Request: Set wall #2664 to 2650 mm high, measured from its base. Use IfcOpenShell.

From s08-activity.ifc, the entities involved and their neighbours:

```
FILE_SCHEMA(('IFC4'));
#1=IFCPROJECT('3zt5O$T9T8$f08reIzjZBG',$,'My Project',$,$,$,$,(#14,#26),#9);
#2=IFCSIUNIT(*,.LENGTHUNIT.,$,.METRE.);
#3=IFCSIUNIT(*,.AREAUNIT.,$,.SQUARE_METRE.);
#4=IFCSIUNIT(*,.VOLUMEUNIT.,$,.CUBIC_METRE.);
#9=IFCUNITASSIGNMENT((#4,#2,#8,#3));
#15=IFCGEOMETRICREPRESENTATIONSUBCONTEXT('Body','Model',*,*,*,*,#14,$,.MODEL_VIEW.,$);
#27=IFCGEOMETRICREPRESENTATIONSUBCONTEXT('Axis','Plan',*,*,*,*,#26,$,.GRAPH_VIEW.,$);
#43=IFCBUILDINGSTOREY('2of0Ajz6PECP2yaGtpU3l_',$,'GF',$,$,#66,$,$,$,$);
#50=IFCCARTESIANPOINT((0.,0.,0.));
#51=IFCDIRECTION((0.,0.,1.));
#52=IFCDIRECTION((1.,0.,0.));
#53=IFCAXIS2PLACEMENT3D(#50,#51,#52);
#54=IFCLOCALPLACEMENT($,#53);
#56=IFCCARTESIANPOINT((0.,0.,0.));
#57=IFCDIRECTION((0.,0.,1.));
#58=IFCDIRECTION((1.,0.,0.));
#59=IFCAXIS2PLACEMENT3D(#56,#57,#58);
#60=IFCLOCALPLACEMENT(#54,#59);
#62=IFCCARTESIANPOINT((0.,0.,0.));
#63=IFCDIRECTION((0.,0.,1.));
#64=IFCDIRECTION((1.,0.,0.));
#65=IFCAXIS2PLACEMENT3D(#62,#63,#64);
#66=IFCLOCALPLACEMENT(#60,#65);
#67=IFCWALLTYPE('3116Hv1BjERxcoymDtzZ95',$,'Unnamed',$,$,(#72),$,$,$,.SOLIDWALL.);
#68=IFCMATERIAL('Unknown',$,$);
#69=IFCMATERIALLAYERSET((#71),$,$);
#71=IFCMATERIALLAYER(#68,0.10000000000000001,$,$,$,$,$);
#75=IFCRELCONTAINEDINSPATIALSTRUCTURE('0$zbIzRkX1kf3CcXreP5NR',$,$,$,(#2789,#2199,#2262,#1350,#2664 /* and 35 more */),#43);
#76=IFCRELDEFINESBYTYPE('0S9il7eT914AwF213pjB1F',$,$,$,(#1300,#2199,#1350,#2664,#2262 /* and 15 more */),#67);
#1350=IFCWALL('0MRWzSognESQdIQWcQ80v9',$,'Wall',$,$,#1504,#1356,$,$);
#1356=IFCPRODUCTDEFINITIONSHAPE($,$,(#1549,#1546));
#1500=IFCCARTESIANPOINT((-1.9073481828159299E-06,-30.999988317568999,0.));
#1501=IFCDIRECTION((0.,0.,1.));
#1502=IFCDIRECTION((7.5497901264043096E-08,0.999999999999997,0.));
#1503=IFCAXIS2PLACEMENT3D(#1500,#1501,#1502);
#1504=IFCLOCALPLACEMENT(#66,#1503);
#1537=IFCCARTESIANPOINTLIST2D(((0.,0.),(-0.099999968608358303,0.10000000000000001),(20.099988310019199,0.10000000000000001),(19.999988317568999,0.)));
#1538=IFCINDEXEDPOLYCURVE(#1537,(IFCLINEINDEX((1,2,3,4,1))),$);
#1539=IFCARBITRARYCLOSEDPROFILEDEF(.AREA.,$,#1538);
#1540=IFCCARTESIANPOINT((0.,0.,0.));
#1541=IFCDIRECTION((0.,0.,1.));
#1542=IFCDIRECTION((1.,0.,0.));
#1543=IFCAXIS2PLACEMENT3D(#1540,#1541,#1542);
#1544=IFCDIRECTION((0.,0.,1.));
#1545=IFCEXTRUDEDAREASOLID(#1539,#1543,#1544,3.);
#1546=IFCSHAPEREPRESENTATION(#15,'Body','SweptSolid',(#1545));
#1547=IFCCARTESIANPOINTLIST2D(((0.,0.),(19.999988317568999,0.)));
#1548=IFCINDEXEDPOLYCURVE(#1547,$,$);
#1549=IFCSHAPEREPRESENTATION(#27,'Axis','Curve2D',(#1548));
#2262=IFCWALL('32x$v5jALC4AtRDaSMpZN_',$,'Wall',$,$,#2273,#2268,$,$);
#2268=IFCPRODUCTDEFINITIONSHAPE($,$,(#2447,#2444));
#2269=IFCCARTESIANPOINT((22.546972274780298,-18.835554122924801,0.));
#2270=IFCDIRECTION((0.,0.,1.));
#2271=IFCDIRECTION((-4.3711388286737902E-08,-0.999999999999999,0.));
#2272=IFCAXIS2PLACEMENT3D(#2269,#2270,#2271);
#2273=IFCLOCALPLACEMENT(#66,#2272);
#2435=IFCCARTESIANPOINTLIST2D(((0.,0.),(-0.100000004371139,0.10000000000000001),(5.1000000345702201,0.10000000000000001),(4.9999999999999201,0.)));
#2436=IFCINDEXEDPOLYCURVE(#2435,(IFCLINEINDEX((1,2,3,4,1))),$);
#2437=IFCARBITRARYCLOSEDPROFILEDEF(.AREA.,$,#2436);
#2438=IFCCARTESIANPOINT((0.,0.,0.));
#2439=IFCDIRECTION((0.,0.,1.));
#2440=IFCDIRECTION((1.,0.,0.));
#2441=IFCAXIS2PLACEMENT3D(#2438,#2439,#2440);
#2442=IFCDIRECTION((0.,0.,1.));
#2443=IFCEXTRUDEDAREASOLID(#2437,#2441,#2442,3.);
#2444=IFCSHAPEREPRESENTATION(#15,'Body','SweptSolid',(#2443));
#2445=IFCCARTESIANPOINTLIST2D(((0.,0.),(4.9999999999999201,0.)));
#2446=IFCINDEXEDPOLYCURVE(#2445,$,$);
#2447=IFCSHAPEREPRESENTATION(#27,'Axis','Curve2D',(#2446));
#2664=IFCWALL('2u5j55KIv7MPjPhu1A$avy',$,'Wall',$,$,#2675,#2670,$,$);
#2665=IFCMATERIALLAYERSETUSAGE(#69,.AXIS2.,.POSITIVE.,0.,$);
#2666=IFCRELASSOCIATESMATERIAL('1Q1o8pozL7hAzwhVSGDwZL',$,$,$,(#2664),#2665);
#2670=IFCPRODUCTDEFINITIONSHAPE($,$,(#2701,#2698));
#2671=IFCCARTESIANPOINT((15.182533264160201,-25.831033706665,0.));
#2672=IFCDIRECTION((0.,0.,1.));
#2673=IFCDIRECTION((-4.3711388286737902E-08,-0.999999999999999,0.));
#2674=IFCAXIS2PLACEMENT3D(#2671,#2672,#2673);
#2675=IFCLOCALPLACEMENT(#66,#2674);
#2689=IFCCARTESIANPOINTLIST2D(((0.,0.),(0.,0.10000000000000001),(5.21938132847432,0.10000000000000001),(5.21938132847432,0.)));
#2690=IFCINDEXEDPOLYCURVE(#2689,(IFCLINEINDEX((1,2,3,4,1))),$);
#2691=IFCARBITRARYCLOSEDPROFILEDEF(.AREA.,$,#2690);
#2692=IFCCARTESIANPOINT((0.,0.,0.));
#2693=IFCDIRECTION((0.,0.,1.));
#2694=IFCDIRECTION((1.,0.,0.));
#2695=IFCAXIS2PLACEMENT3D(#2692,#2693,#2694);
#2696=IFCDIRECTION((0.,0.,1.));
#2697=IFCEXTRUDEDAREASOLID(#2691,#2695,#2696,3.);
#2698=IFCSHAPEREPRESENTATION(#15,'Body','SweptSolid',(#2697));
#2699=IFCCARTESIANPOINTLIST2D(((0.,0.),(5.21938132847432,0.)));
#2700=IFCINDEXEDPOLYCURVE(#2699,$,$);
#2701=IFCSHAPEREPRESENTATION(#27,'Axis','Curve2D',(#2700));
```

```python
import ifcopenshell
import ifcopenshell.geom
import ifcopenshell.util.representation
import ifcopenshell.util.shape
import ifcopenshell.util.unit

model = ifcopenshell.open("s08-activity.ifc")
unit_scale = ifcopenshell.util.unit.calculate_unit_scale(model)
settings = ifcopenshell.geom.settings()


def volume(element):
    """Net volume in cubic metres, openings subtracted."""
    shape = ifcopenshell.geom.create_shape(settings, element)
    return ifcopenshell.util.shape.get_volume(shape.geometry)


wall = model.by_guid("2u5j55KIv7MPjPhu1A$avy")
before = volume(wall)

body = ifcopenshell.util.representation.get_representation(wall, "Model", "Body")
solid = body.Items[0]
old_height = solid.Depth
solid.Depth = 2.65 / unit_scale
after = volume(wall)

print(f"height {old_height:g} -> {solid.Depth:g}, volume {before:.3f} -> {after:.3f} m3")

model.write("s08-activity_updated.ifc")
```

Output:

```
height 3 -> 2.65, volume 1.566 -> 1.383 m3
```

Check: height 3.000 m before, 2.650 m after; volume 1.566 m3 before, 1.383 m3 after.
